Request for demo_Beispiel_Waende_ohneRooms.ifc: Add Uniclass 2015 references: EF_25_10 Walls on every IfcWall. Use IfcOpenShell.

First a look at what the model holds.

```python
import ifcopenshell

model = ifcopenshell.open("demo_Beispiel_Waende_ohneRooms.ifc")
print(model.schema)
print("classifications:", [c.Name for c in model.by_type("IfcClassification")])
for ifc_class in ("IfcDoor", "IfcRoof", "IfcStair", "IfcWall", "IfcWindow"):
    print(ifc_class, len(model.by_type(ifc_class)))
```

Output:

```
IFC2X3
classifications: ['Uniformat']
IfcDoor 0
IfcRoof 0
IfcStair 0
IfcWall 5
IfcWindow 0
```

```python
import ifcopenshell
import ifcopenshell.api.classification

model = ifcopenshell.open("demo_Beispiel_Waende_ohneRooms.ifc")

# IFC2X3 requires Source and Edition and has no link from the project to the system.
system = model.create_entity("IfcClassification", Source="NBS", Edition="2015", Name="Uniclass 2015")

codes = {
    "IfcWall": ("EF_25_10", "Walls"),
}
for ifc_class, (code, name) in codes.items():
    products = model.by_type(ifc_class)
    ifcopenshell.api.classification.add_reference(
        model, products=products, classification=system, identification=code, name=name
    )
    print(code, len(products))

model.write("demo_Beispiel_Waende_ohneRooms_v2.ifc")
```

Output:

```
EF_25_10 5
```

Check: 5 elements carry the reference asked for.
